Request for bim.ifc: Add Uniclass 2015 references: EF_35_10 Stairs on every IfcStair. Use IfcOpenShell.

First a look at what the model holds.

```python
import ifcopenshell

model = ifcopenshell.open("bim.ifc")
print(model.schema)
print("classifications:", [c.Name for c in model.by_type("IfcClassification")])
for ifc_class in ("IfcDoor", "IfcRoof", "IfcStair", "IfcWall", "IfcWindow"):
    print(ifc_class, len(model.by_type(ifc_class)))
```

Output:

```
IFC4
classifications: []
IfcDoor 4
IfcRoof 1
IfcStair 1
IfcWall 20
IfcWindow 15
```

```python
import ifcopenshell
import ifcopenshell.api.classification

model = ifcopenshell.open("bim.ifc")

system = ifcopenshell.api.classification.add_classification(model, classification="Uniclass 2015")

codes = {
    "IfcStair": ("EF_35_10", "Stairs"),
}
for ifc_class, (code, name) in codes.items():
    products = model.by_type(ifc_class)
    ifcopenshell.api.classification.add_reference(
        model, products=products, classification=system, identification=code, name=name
    )
    print(code, len(products))

model.write("bim_updated.ifc")
```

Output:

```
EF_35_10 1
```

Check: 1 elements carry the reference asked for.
